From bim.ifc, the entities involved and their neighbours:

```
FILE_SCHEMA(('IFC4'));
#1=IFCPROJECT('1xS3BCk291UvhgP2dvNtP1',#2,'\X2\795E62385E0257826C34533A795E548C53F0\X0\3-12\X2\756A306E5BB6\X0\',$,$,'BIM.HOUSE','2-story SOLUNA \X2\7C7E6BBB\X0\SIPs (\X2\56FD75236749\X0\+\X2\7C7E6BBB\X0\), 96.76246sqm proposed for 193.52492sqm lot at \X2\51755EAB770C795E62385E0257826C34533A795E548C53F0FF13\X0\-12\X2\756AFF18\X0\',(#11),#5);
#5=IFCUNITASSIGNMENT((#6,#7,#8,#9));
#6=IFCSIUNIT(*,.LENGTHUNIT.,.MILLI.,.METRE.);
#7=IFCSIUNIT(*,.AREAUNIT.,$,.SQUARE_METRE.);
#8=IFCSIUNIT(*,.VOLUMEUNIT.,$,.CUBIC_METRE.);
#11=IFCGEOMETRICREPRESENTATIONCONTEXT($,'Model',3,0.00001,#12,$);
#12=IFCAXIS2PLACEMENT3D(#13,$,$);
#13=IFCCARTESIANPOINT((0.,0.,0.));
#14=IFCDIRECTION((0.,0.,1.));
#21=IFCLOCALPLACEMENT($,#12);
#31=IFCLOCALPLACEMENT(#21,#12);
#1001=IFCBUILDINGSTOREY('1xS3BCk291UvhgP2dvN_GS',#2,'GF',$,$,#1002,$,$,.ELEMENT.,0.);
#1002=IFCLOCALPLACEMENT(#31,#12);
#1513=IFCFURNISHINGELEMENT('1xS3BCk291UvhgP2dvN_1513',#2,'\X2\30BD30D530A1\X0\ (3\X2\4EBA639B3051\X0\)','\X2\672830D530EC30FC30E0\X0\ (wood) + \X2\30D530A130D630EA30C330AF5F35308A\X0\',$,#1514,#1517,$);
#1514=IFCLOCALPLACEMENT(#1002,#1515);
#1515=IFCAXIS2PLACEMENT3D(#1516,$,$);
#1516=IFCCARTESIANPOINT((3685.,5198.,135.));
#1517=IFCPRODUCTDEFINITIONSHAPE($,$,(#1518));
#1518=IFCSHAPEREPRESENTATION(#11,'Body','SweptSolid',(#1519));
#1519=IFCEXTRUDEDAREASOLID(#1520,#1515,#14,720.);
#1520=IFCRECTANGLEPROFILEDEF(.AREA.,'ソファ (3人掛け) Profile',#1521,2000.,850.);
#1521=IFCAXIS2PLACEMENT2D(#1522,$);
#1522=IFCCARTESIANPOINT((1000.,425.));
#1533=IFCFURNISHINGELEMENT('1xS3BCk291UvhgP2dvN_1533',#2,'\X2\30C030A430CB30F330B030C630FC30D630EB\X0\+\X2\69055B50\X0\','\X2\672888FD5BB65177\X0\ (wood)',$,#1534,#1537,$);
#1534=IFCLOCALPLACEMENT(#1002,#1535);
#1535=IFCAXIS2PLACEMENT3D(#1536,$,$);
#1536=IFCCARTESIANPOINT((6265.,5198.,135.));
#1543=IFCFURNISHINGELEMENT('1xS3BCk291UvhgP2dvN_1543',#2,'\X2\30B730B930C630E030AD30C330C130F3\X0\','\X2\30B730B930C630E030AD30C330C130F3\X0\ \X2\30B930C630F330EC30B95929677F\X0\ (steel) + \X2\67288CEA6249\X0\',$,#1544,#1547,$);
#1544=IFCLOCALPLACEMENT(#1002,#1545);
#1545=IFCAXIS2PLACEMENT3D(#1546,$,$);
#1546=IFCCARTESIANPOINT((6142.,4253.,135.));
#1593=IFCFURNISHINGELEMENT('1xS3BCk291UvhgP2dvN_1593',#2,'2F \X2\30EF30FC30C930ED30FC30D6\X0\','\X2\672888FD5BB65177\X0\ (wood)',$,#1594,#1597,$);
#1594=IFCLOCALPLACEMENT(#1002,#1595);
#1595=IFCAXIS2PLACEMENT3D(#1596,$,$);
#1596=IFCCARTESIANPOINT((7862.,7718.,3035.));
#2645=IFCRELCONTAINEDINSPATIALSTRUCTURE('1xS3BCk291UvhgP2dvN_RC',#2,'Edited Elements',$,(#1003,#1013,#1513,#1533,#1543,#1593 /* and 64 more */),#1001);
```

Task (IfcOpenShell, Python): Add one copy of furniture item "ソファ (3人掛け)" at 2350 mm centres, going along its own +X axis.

```python
import ifcopenshell
import ifcopenshell.api.geometry
import ifcopenshell.api.root
import ifcopenshell.util.element
import ifcopenshell.util.placement
import ifcopenshell.util.unit

model = ifcopenshell.open("bim.ifc")
unit_scale = ifcopenshell.util.unit.calculate_unit_scale(model)


def reuse_history(source, copy):
    """copy_class also copies each property set's owner history, people and application; keep the originals."""
    for rel in copy.IsDefinedBy:
        if rel.is_a("IfcRelDefinesByProperties") and (history := rel.RelatingPropertyDefinition.OwnerHistory):
            rel.RelatingPropertyDefinition.OwnerHistory = source.OwnerHistory
            ifcopenshell.util.element.remove_deep2(model, history)


source = model.by_guid("1xS3BCk291UvhgP2dvN_1513")
base = ifcopenshell.util.placement.get_local_placement(source.ObjectPlacement)
step = base[:3, 0] * 2.35 / unit_scale

for i in range(1, 2):
    copy = ifcopenshell.api.root.copy_class(model, product=source)
    copy.Representation = ifcopenshell.util.element.copy_deep(
        model, source.Representation, exclude=["IfcGeometricRepresentationContext", "IfcRepresentationMap"]
    )
    reuse_history(source, copy)
    matrix = base.copy()
    matrix[:3, 3] += i * step
    print("added at", matrix[:3, 3].round(3) + 0.0)
    ifcopenshell.api.geometry.edit_object_placement(model, product=copy, matrix=matrix, is_si=False)

model.write("bim_updated.ifc")
```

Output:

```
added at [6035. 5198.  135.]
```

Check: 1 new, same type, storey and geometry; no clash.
